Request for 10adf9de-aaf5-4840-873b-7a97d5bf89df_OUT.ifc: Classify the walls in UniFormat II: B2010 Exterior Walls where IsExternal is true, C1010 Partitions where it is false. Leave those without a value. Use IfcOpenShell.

First a look at what the model holds.

```python
import ifcopenshell
import ifcopenshell.util.element

model = ifcopenshell.open("10adf9de-aaf5-4840-873b-7a97d5bf89df_OUT.ifc")
print(model.schema)
print("classifications:", [c.Name for c in model.by_type("IfcClassification")])
values = [ifcopenshell.util.element.get_pset(e, "Pset_WallCommon", "IsExternal") for e in model.by_type("IfcWall")]
for value in (True, False, None):
    print("IsExternal", value, values.count(value))
```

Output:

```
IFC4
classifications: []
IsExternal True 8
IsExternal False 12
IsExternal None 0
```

```python
import ifcopenshell
import ifcopenshell.api.classification
import ifcopenshell.util.element

model = ifcopenshell.open("10adf9de-aaf5-4840-873b-7a97d5bf89df_OUT.ifc")

system = ifcopenshell.api.classification.add_classification(model, classification="UniFormat II")

walls = model.by_type("IfcWall")
external = {e: ifcopenshell.util.element.get_pset(e, "Pset_WallCommon", "IsExternal") for e in walls}
for flag, code, name in ((True, "B2010", "Exterior Walls"), (False, "C1010", "Partitions")):
    products = [e for e in walls if external[e] is flag]
    ifcopenshell.api.classification.add_reference(
        model, products=products, classification=system, identification=code, name=name
    )
    print(code, len(products))

model.write("10adf9de-aaf5-4840-873b-7a97d5bf89df_OUT_v2.ifc")
```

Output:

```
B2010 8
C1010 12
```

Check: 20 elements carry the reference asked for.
